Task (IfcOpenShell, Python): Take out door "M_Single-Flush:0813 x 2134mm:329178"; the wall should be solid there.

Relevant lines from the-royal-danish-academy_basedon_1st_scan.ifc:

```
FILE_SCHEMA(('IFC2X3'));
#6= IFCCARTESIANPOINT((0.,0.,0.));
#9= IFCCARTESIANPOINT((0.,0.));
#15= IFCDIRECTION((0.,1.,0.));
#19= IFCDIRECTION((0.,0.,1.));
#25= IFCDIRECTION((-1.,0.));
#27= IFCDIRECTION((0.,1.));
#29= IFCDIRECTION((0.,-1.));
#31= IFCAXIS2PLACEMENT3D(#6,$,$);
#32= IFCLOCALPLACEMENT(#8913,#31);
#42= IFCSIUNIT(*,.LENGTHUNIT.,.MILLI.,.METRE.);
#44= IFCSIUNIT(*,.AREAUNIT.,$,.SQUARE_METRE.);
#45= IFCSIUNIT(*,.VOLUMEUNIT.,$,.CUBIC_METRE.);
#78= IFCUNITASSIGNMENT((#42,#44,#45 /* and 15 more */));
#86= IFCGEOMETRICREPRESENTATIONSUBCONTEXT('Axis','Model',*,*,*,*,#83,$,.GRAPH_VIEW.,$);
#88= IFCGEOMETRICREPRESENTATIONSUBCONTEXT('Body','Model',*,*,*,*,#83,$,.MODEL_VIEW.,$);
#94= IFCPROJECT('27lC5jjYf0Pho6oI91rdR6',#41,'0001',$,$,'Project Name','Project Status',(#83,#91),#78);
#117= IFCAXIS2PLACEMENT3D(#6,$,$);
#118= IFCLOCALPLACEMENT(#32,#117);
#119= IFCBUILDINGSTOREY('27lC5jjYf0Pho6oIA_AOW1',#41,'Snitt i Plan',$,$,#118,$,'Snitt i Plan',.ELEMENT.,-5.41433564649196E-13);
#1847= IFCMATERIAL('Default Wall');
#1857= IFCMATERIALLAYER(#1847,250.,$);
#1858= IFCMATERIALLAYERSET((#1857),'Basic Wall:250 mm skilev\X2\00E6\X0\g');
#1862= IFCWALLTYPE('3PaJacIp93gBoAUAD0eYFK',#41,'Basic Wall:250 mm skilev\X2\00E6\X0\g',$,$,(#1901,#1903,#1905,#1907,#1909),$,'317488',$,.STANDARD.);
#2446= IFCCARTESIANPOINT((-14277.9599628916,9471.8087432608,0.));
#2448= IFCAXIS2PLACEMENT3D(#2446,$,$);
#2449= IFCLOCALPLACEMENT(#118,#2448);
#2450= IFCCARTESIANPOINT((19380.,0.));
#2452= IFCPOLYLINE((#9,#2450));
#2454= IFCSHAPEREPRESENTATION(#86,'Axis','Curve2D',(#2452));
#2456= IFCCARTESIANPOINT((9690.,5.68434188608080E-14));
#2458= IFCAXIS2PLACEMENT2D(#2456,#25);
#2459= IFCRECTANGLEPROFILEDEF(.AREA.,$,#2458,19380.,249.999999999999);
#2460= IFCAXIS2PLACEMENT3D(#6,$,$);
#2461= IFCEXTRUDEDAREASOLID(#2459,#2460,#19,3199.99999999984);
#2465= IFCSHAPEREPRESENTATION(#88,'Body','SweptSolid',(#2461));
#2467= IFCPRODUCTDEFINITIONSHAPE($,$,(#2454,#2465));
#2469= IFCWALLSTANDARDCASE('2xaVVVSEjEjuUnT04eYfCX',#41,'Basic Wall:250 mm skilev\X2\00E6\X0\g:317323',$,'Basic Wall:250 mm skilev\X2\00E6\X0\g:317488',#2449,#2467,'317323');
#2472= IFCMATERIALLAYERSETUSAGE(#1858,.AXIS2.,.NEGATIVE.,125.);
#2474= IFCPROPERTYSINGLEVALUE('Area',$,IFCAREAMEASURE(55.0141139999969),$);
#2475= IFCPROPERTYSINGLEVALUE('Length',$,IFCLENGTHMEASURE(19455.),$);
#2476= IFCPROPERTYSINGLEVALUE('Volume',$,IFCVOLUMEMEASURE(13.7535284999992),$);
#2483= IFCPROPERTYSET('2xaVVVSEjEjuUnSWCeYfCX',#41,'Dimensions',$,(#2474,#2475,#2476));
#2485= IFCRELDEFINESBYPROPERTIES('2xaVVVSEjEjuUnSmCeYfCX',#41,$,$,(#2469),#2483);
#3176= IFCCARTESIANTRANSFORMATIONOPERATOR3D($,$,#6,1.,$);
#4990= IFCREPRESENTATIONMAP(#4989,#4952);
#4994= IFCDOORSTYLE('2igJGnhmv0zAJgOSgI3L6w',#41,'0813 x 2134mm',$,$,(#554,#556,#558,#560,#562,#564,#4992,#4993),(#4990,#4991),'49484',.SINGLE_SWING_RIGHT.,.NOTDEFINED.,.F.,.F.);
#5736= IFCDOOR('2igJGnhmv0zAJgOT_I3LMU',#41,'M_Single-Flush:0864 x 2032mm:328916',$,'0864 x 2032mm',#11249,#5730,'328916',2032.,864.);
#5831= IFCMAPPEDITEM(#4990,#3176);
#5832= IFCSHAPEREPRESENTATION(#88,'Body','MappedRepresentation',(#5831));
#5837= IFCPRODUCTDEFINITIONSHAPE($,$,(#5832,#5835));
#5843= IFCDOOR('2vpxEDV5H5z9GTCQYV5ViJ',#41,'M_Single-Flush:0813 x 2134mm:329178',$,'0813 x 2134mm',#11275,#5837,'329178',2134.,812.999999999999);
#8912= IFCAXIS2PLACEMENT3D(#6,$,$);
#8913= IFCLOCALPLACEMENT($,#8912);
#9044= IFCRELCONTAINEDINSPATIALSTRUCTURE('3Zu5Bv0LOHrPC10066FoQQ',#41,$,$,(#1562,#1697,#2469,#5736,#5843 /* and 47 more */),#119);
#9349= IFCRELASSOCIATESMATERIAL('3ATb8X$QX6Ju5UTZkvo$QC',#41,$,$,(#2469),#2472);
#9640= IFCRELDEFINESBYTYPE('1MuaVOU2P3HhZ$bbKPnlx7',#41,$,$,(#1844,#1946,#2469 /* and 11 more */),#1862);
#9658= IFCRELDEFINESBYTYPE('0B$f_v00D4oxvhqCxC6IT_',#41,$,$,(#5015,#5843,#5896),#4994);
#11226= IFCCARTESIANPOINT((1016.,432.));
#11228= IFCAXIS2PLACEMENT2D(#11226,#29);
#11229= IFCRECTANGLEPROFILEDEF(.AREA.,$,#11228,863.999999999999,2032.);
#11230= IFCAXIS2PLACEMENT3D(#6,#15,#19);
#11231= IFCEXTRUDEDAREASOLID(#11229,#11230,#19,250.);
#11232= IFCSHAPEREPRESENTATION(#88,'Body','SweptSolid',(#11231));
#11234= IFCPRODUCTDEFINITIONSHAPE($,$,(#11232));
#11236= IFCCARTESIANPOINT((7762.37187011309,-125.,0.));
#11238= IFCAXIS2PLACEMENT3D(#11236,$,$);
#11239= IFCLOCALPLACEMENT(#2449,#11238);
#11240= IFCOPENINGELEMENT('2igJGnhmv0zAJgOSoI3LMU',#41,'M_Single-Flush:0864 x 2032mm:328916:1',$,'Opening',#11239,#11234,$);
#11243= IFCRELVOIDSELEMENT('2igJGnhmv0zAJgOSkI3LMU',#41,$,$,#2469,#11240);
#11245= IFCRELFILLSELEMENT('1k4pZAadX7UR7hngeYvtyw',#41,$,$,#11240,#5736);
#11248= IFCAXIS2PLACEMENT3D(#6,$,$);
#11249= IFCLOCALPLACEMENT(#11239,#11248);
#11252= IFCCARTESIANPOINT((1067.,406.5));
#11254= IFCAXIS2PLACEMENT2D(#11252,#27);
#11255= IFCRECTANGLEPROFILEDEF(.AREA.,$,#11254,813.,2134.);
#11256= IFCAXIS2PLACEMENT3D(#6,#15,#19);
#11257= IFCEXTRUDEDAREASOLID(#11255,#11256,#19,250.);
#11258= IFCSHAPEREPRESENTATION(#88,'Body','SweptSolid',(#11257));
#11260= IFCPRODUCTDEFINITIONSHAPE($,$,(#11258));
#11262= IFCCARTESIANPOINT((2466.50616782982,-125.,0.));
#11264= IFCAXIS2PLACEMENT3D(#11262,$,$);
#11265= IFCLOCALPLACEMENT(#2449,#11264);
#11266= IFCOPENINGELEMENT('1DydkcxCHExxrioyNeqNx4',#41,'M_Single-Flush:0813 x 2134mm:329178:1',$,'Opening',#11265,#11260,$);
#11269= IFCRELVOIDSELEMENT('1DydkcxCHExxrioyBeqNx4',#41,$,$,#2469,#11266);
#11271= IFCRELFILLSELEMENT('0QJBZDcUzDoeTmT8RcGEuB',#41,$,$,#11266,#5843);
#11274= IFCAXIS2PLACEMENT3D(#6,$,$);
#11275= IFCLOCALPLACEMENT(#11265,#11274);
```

```python
import ifcopenshell
import ifcopenshell.api.feature
import ifcopenshell.api.pset
import ifcopenshell.api.root
import ifcopenshell.geom
import ifcopenshell.util.element
import ifcopenshell.util.shape
import ifcopenshell.util.unit

model = ifcopenshell.open("the-royal-danish-academy_basedon_1st_scan.ifc")
area_scale = ifcopenshell.util.unit.calculate_unit_scale(model, "AREAUNIT")
volume_scale = ifcopenshell.util.unit.calculate_unit_scale(model, "VOLUMEUNIT")
settings = ifcopenshell.geom.settings()


def volume(element):
    """Net volume in cubic metres, openings subtracted."""
    shape = ifcopenshell.geom.create_shape(settings, element)
    return ifcopenshell.util.shape.get_volume(shape.geometry)


door = model.by_id(5843)
opening = door.FillsVoids[0].RelatingOpeningElement
wall = opening.VoidsElements[0].RelatingBuildingElement
before = volume(wall)

ifcopenshell.api.root.remove_product(model, product=door)
ifcopenshell.api.feature.remove_feature(model, feature=opening)

after = volume(wall)
thickness = 0.25  # wall thickness in metres

# Update the wall's stored quantities.
pset = model.by_id(ifcopenshell.util.element.get_pset(wall, "Dimensions", should_inherit=False)["id"])
ifcopenshell.api.pset.edit_pset(model, pset=pset, properties={
    "Area": model.create_entity("IfcAreaMeasure", after / thickness / area_scale),
    "Volume": model.create_entity("IfcVolumeMeasure", after / volume_scale),
})

print(f"wall volume {before:.3f} -> {after:.3f} m3")

model.write("the-royal-danish-academy_basedon_1st_scan_updated.ifc")
```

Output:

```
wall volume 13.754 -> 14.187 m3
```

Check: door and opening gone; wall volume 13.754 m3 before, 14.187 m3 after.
